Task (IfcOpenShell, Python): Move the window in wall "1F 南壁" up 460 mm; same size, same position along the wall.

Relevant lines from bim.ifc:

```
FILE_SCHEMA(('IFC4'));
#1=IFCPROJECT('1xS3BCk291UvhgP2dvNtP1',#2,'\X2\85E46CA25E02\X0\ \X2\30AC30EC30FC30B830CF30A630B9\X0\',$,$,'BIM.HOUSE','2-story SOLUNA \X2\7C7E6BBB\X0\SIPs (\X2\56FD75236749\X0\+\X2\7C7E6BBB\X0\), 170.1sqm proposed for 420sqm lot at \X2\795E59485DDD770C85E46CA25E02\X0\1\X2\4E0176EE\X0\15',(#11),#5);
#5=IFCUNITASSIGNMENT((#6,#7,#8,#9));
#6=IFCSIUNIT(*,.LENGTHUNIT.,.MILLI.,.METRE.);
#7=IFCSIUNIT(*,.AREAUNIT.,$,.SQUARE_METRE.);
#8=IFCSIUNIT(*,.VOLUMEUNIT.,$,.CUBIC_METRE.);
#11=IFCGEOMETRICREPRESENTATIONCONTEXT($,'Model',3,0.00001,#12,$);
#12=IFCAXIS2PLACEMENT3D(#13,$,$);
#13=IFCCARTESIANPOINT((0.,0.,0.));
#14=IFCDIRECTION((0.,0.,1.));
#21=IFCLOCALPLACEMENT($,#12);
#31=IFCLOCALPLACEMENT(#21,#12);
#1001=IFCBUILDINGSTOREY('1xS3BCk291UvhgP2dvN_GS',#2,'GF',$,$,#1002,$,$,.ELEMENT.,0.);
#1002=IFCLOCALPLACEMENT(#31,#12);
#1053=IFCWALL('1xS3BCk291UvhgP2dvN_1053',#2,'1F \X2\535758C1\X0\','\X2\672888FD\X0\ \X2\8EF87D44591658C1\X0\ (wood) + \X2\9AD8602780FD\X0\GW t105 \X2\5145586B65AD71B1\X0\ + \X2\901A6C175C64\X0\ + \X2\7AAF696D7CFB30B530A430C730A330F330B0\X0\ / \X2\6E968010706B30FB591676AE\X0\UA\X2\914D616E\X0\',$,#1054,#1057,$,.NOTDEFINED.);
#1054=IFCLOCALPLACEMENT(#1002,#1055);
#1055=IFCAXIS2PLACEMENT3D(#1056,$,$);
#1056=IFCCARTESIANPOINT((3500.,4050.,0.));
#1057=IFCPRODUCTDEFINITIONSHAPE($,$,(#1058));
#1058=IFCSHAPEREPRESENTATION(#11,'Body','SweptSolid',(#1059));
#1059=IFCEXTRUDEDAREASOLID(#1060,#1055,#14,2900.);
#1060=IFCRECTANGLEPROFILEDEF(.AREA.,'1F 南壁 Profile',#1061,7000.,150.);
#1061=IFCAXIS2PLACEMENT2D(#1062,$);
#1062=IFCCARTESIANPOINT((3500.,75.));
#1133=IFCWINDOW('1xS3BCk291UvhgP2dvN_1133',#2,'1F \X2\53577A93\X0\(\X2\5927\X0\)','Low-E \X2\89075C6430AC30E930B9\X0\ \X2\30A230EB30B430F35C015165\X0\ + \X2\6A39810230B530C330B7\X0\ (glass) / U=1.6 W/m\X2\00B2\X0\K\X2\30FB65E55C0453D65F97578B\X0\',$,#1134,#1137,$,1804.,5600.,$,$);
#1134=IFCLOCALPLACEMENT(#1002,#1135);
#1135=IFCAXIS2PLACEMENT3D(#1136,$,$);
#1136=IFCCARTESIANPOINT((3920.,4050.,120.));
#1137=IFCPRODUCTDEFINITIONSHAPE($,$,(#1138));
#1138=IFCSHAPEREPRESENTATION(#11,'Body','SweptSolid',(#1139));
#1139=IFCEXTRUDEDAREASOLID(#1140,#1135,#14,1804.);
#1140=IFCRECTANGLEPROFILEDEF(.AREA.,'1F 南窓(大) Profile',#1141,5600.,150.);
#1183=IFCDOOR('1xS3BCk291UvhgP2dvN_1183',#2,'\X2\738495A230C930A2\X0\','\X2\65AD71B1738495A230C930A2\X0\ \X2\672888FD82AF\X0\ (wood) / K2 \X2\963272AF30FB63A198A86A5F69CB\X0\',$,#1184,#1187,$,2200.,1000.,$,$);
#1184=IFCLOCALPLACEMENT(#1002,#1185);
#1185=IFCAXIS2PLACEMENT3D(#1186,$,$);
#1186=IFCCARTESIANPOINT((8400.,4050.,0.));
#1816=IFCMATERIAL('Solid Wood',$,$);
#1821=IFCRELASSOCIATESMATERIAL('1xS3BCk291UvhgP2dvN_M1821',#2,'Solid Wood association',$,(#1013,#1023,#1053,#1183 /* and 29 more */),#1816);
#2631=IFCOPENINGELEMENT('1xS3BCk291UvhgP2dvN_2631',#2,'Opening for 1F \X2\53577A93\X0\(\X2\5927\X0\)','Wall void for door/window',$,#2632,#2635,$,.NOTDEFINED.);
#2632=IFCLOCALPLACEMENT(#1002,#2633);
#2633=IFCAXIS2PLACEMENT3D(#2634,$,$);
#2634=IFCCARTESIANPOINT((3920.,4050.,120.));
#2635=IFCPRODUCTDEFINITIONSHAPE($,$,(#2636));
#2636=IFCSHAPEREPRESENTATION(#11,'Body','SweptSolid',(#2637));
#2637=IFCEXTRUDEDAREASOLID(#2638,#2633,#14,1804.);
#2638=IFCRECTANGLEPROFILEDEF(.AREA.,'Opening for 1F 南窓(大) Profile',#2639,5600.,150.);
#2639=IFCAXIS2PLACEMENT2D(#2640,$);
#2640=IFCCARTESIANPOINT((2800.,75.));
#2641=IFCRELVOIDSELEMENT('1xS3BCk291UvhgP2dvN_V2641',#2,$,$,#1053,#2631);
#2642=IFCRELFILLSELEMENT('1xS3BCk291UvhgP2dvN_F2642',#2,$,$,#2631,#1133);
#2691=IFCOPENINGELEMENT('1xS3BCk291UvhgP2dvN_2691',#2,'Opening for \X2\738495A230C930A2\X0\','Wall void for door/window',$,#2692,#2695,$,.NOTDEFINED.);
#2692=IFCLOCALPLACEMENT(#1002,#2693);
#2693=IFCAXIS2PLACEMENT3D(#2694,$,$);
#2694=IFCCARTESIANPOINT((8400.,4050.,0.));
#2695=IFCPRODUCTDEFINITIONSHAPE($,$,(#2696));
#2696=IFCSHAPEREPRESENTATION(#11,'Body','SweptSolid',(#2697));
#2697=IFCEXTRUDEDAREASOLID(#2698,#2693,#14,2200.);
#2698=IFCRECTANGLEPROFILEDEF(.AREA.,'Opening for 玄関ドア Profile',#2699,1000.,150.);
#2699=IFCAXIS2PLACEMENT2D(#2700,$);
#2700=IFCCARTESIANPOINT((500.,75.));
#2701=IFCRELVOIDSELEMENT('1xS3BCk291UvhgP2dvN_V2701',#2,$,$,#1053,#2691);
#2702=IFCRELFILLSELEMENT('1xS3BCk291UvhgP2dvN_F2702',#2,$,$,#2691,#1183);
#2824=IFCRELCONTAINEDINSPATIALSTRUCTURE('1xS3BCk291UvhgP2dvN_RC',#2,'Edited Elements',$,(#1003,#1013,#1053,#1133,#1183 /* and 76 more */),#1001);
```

```python
import numpy as np
import ifcopenshell
import ifcopenshell.api.geometry
import ifcopenshell.util.placement
import ifcopenshell.util.unit

model = ifcopenshell.open("bim.ifc")
unit_scale = ifcopenshell.util.unit.calculate_unit_scale(model)

window = model.by_id(1133)
opening = window.FillsVoids[0].RelatingOpeningElement
dz = 0.46 / unit_scale

shift = np.array([0.0, 0.0, dz])
# The window is not placed relative to its opening, so move both.
for product in (opening, window):
    matrix = ifcopenshell.util.placement.get_local_placement(product.ObjectPlacement)
    matrix[:3, 3] += shift
    ifcopenshell.api.geometry.edit_object_placement(model, product=product, matrix=matrix, is_si=False)

print(f"moved by {dz * unit_scale:+.3f} m")

model.write("bim_rev.ifc")
```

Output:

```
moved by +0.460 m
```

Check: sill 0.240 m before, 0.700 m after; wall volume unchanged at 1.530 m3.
